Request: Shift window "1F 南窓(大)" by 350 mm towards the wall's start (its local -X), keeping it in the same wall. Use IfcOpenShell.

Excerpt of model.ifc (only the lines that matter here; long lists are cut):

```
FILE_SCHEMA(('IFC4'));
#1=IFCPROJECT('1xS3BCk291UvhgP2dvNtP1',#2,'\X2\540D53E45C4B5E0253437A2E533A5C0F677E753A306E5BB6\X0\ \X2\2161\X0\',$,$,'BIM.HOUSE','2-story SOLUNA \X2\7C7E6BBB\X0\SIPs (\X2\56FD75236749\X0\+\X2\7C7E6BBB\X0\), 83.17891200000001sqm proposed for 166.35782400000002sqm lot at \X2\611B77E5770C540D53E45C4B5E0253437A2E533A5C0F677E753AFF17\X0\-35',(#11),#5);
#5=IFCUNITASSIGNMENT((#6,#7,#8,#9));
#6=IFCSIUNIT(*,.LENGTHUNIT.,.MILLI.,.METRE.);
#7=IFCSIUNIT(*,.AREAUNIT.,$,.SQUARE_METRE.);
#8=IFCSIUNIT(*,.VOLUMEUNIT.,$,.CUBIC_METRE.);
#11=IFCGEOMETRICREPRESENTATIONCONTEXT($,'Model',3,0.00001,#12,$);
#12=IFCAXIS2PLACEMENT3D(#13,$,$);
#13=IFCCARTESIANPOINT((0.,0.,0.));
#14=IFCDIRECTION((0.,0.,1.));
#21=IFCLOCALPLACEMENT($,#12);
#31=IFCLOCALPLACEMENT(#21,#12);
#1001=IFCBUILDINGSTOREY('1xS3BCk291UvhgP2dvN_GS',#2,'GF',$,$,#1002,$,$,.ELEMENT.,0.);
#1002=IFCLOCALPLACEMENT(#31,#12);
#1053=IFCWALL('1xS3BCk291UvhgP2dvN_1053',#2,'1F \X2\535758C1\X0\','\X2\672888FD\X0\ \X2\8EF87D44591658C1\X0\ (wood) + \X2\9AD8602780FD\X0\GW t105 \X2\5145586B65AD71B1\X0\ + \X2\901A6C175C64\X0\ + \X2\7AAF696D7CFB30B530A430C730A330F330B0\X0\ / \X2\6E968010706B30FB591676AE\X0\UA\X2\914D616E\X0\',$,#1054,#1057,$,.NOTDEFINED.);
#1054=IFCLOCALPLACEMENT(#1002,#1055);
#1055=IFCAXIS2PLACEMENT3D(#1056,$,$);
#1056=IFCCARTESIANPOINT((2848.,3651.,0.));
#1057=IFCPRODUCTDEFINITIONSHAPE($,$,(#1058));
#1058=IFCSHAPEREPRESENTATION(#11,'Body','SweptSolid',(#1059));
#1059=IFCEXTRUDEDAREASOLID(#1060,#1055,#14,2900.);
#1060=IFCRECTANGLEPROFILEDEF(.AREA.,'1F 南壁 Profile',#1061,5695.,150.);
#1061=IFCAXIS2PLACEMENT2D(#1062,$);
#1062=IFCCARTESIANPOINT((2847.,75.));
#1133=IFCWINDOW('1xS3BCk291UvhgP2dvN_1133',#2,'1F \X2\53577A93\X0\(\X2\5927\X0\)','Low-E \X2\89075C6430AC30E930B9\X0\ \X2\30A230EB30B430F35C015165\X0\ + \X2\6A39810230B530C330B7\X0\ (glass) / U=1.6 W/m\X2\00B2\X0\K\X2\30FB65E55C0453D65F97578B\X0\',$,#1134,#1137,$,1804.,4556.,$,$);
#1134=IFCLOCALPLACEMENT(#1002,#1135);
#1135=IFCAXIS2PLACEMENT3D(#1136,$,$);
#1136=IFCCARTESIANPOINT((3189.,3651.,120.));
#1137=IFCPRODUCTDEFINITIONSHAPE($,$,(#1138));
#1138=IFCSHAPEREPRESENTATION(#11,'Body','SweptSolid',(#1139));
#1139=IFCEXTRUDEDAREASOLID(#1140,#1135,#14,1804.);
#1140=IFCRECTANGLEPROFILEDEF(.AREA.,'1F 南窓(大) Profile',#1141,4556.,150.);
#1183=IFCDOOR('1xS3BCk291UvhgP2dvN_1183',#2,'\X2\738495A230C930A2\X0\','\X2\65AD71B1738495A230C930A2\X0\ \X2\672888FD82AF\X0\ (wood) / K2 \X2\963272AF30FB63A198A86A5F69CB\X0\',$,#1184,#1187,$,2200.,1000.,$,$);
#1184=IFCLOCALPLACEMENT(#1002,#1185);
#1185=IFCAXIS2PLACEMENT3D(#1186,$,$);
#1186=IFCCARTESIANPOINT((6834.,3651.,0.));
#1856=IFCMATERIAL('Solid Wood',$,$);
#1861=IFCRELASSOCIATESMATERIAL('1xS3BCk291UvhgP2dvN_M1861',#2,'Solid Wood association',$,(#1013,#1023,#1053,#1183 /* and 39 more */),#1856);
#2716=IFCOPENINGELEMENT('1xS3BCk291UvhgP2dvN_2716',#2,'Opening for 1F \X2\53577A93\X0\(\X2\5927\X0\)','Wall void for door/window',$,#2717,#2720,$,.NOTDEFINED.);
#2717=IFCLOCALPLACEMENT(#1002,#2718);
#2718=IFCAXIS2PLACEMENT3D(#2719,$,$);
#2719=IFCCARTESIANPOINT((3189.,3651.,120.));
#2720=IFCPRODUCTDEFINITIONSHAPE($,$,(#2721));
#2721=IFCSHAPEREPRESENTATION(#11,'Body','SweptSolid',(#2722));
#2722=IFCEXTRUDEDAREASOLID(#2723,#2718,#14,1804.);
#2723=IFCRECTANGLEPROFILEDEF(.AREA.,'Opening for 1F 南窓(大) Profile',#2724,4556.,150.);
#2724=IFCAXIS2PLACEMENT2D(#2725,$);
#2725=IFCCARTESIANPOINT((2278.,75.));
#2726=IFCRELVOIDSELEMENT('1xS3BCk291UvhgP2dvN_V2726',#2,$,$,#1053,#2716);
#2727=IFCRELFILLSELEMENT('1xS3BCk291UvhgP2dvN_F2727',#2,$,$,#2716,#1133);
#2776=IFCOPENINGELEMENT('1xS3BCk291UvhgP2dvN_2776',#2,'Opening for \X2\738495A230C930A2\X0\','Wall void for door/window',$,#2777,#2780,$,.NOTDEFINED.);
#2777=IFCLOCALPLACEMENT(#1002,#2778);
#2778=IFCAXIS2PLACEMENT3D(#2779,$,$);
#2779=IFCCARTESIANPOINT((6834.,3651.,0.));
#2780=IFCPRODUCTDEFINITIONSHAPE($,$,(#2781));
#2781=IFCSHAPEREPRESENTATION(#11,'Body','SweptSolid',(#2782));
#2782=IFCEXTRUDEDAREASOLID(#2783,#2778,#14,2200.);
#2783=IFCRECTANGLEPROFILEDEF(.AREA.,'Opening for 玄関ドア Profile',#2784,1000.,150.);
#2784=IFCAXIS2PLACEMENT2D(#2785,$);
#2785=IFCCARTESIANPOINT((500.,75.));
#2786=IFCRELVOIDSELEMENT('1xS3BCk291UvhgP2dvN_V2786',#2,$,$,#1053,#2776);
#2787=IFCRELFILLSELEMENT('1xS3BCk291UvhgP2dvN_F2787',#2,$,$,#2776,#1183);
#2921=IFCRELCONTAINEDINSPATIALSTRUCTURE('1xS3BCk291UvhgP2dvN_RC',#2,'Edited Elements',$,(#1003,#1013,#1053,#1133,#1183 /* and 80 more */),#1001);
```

```python
import ifcopenshell
import ifcopenshell.api.geometry
import ifcopenshell.util.placement
import ifcopenshell.util.unit

model = ifcopenshell.open("model.ifc")
unit_scale = ifcopenshell.util.unit.calculate_unit_scale(model)

window = model.by_guid("1xS3BCk291UvhgP2dvN_1133")
opening = window.FillsVoids[0].RelatingOpeningElement
wall = opening.VoidsElements[0].RelatingBuildingElement

wall_matrix = ifcopenshell.util.placement.get_local_placement(wall.ObjectPlacement)
shift = wall_matrix[:3, 0] * -0.35 / unit_scale
before = ifcopenshell.util.placement.get_local_placement(window.ObjectPlacement)[:3, 3].copy()

# The window is not placed relative to its opening, so move both.
for product in (opening, window):
    matrix = ifcopenshell.util.placement.get_local_placement(product.ObjectPlacement)
    matrix[:3, 3] += shift
    ifcopenshell.api.geometry.edit_object_placement(model, product=product, matrix=matrix, is_si=False)

after = ifcopenshell.util.placement.get_local_placement(window.ObjectPlacement)[:3, 3]
print("window moved by", (after - before).round(3) + 0.0)

model.write("model_v2.ifc")
```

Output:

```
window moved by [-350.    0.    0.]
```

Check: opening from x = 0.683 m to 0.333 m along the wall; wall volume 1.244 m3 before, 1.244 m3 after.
